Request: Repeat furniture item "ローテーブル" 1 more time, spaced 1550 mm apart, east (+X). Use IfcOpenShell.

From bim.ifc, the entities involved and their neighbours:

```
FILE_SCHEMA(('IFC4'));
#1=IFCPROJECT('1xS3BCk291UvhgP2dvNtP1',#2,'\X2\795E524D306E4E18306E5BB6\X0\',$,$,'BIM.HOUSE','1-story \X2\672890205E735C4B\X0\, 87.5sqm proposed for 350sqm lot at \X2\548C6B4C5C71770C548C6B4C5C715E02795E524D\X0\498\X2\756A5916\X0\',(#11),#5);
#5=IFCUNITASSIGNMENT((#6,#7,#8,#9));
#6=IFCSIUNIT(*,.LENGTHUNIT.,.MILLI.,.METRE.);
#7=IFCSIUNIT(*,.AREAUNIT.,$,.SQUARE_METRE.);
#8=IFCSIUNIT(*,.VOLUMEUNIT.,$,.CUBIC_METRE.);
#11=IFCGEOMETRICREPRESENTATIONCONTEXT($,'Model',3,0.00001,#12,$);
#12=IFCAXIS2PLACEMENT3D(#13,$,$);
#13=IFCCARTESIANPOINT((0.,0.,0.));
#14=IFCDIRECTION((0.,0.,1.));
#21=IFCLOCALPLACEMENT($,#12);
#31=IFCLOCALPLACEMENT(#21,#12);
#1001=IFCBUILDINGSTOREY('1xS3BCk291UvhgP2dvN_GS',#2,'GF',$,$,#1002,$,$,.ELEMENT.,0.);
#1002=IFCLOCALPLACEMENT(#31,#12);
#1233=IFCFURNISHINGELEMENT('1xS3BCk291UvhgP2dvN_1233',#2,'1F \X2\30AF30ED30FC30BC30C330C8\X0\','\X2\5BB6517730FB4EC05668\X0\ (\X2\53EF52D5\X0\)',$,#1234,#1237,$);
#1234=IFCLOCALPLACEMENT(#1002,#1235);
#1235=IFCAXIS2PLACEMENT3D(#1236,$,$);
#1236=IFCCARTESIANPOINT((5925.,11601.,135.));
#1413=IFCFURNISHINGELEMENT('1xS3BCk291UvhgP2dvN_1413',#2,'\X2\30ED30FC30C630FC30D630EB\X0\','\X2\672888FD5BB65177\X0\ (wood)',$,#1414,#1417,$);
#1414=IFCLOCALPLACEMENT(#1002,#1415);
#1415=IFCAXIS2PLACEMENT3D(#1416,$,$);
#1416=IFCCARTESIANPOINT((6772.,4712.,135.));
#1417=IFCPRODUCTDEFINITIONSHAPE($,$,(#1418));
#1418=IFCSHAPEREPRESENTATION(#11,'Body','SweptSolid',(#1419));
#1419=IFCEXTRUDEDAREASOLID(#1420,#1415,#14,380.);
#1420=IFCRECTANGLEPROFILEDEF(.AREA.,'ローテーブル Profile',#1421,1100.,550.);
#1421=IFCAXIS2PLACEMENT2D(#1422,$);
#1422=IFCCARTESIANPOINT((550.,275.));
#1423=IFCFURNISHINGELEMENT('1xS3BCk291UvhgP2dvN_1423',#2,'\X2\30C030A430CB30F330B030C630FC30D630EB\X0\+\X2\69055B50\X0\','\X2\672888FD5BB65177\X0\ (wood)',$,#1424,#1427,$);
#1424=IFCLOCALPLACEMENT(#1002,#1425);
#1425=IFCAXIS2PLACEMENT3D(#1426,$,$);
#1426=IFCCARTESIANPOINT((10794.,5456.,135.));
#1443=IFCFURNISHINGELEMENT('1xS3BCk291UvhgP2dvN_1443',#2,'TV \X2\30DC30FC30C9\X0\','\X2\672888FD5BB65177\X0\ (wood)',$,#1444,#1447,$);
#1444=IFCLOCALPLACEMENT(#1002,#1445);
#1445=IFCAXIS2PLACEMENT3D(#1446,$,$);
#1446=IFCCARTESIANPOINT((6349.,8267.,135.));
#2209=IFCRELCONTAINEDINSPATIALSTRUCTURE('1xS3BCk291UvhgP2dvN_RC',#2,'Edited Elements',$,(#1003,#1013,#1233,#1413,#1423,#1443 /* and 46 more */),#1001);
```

```python
import numpy as np
import ifcopenshell
import ifcopenshell.api.geometry
import ifcopenshell.api.root
import ifcopenshell.util.element
import ifcopenshell.util.placement
import ifcopenshell.util.unit

model = ifcopenshell.open("bim.ifc")
unit_scale = ifcopenshell.util.unit.calculate_unit_scale(model)


def reuse_history(source, copy):
    """copy_class also copies each property set's owner history, people and application; keep the originals."""
    for rel in copy.IsDefinedBy:
        if rel.is_a("IfcRelDefinesByProperties") and (history := rel.RelatingPropertyDefinition.OwnerHistory):
            rel.RelatingPropertyDefinition.OwnerHistory = source.OwnerHistory
            ifcopenshell.util.element.remove_deep2(model, history)


source = model.by_guid("1xS3BCk291UvhgP2dvN_1413")
base = ifcopenshell.util.placement.get_local_placement(source.ObjectPlacement)
step = np.array([1.0, 0.0, 0.0]) * 1.55 / unit_scale

for i in range(1, 2):
    copy = ifcopenshell.api.root.copy_class(model, product=source)
    copy.Representation = ifcopenshell.util.element.copy_deep(
        model, source.Representation, exclude=["IfcGeometricRepresentationContext", "IfcRepresentationMap"]
    )
    reuse_history(source, copy)
    matrix = base.copy()
    matrix[:3, 3] += i * step
    print("added at", matrix[:3, 3].round(3) + 0.0)
    ifcopenshell.api.geometry.edit_object_placement(model, product=copy, matrix=matrix, is_si=False)

model.write("bim_edited.ifc")
```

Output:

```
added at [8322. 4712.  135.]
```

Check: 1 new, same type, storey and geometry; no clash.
